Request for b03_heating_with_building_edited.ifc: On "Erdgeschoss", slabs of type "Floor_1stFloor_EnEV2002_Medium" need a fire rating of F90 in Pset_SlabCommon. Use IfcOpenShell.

First a look at what the model holds.

```python
import ifcopenshell
import ifcopenshell.util.element

model = ifcopenshell.open("b03_heating_with_building_edited.ifc")
print(model.schema)
storey = next(s for s in model.by_type("IfcBuildingStorey") if s.Name == "Erdgeschoss")
slabs = [e for e in ifcopenshell.util.element.get_decomposition(storey) if e.is_a("IfcSlab")]
seen = {}
for e in slabs:
    element_type = ifcopenshell.util.element.get_type(e)
    key = (element_type.Name if element_type != e and element_type else None, ifcopenshell.util.element.get_pset(e, "Pset_SlabCommon", "FireRating"))
    seen[key] = seen.get(key, 0) + 1
for (name, value), count in sorted(seen.items(), key=str):
    print(count, "x", name, "|", value)
```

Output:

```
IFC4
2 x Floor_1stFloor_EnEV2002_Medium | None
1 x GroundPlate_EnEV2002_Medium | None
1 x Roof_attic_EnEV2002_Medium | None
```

```python
import ifcopenshell
import ifcopenshell.api.pset
import ifcopenshell.util.element

model = ifcopenshell.open("b03_heating_with_building_edited.ifc")

storey = next(s for s in model.by_type("IfcBuildingStorey") if s.Name == "Erdgeschoss")
slabs = [e for e in ifcopenshell.util.element.get_decomposition(storey) if e.is_a("IfcSlab")]

count = 0
for e in slabs:
    element_type = ifcopenshell.util.element.get_type(e)
    if element_type in (None, e) or element_type.Name != "Floor_1stFloor_EnEV2002_Medium":
        continue
    found = ifcopenshell.util.element.get_pset(e, "Pset_SlabCommon", should_inherit=False)
    if found:
        pset = model.by_id(found["id"])
        if len(ifcopenshell.util.element.get_elements_by_pset(pset)) > 1:
            pset = ifcopenshell.api.pset.unshare_pset(model, products=[e], pset=pset)[0]
    else:
        pset = ifcopenshell.api.pset.add_pset(model, product=e, name="Pset_SlabCommon")
    ifcopenshell.api.pset.edit_pset(model, pset=pset, properties={"FireRating": "F90"})
    count += 1

print(count, "slabs updated")

model.write("b03_heating_with_building_edited_edited.ifc")
```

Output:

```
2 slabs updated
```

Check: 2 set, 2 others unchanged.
